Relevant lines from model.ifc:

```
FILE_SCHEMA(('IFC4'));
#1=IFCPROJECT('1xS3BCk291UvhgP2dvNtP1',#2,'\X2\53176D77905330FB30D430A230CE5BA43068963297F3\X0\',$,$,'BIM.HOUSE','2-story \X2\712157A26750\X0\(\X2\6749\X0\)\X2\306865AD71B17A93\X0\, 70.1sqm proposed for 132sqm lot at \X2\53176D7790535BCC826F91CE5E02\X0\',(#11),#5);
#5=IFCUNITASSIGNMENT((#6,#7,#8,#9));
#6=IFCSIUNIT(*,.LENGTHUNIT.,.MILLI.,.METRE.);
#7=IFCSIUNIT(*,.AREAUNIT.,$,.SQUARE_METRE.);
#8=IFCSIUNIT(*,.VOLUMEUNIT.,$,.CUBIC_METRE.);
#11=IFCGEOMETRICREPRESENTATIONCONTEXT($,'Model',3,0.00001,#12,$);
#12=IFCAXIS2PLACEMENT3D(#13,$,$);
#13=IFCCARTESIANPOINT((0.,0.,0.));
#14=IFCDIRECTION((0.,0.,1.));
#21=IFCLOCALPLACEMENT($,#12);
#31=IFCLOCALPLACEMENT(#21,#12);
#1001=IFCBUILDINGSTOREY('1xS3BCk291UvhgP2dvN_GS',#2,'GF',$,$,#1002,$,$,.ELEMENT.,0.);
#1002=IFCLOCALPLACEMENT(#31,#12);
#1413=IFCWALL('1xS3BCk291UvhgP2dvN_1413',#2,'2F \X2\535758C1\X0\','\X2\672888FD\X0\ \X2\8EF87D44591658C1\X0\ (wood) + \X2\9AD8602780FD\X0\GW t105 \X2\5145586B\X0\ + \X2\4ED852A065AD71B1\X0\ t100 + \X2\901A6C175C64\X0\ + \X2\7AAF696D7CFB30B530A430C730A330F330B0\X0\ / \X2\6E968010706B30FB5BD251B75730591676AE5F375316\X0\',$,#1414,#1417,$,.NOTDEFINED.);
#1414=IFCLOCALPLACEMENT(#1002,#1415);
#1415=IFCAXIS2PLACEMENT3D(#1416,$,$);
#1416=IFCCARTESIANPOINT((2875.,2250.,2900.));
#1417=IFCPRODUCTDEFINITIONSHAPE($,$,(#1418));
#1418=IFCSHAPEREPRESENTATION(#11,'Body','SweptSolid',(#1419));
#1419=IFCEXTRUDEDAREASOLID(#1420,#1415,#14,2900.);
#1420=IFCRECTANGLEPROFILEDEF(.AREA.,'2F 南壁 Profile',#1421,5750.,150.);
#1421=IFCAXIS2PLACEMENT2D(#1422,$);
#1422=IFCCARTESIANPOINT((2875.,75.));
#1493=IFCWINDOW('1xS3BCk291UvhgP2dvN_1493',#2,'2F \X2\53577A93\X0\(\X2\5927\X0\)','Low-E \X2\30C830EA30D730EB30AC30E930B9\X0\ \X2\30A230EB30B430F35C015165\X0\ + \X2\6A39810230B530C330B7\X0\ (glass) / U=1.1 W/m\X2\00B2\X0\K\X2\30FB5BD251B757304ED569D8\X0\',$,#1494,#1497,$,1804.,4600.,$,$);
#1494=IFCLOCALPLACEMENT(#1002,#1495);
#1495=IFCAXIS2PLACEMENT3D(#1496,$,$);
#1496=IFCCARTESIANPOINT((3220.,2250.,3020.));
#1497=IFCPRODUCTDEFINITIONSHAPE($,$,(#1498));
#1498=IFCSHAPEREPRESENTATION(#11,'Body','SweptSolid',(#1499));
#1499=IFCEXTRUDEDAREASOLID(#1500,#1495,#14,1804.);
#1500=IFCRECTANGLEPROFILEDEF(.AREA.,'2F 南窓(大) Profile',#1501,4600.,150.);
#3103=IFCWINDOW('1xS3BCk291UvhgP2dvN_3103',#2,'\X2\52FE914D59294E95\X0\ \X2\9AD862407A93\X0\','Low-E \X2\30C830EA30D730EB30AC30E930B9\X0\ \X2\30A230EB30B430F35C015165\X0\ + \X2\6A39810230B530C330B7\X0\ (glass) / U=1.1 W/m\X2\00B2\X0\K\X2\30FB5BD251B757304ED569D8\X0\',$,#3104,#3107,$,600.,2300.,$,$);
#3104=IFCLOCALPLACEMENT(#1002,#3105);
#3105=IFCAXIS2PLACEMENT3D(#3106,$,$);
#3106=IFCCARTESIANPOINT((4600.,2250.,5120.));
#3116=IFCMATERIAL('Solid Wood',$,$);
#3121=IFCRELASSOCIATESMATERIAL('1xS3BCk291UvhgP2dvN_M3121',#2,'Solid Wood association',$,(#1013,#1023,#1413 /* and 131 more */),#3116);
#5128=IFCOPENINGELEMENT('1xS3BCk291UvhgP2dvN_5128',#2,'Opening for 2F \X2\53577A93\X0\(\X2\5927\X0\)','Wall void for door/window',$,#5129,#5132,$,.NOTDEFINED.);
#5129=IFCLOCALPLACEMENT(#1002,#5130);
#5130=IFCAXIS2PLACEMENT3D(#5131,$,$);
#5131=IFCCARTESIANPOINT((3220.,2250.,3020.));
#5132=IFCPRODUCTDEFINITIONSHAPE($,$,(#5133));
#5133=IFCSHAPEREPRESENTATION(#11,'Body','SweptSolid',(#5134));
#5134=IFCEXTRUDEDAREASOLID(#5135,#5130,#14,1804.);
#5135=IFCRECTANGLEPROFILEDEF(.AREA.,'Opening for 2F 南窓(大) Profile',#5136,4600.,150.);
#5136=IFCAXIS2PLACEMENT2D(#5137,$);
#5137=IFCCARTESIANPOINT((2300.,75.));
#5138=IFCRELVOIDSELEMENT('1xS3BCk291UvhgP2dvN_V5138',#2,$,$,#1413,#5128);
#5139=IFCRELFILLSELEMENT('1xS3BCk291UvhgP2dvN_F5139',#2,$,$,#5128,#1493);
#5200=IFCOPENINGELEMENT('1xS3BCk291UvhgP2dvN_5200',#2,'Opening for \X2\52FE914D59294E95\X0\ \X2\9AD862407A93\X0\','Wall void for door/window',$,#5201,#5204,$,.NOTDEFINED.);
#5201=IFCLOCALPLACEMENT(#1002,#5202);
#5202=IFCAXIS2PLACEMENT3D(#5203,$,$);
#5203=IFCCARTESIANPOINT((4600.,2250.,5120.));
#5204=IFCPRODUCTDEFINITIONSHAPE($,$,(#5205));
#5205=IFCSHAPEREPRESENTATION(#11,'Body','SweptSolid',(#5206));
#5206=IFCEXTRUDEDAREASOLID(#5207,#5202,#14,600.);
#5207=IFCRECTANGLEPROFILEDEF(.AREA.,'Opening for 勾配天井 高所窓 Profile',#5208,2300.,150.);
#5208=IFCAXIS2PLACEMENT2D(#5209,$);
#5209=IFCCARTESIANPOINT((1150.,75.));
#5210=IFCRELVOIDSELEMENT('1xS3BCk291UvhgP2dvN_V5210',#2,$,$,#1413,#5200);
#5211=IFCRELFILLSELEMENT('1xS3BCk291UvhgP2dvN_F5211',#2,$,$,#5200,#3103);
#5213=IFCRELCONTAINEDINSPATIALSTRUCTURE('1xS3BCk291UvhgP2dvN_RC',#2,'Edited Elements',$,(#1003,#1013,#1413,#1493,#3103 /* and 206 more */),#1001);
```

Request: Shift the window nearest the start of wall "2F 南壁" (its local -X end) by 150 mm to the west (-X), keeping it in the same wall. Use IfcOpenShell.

```python
import ifcopenshell
import ifcopenshell.api.geometry
import ifcopenshell.util.placement

model = ifcopenshell.open("model.ifc")

window = model.by_guid("1xS3BCk291UvhgP2dvN_1493")
opening = window.FillsVoids[0].RelatingOpeningElement
wall = opening.VoidsElements[0].RelatingBuildingElement

wall_matrix = ifcopenshell.util.placement.get_local_placement(wall.ObjectPlacement)
shift = wall_matrix[:3, 0] * -150.0
before = ifcopenshell.util.placement.get_local_placement(window.ObjectPlacement)[:3, 3].copy()

# The window is not placed relative to its opening, so move both.
for product in (opening, window):
    matrix = ifcopenshell.util.placement.get_local_placement(product.ObjectPlacement)
    matrix[:3, 3] += shift
    ifcopenshell.api.geometry.edit_object_placement(model, product=product, matrix=matrix, is_si=False)

after = ifcopenshell.util.placement.get_local_placement(window.ObjectPlacement)[:3, 3]
print("window moved by", (after - before).round(3) + 0.0)

model.write("model_updated.ifc")
```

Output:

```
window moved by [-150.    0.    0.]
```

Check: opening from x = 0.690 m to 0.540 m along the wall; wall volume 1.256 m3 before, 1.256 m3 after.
